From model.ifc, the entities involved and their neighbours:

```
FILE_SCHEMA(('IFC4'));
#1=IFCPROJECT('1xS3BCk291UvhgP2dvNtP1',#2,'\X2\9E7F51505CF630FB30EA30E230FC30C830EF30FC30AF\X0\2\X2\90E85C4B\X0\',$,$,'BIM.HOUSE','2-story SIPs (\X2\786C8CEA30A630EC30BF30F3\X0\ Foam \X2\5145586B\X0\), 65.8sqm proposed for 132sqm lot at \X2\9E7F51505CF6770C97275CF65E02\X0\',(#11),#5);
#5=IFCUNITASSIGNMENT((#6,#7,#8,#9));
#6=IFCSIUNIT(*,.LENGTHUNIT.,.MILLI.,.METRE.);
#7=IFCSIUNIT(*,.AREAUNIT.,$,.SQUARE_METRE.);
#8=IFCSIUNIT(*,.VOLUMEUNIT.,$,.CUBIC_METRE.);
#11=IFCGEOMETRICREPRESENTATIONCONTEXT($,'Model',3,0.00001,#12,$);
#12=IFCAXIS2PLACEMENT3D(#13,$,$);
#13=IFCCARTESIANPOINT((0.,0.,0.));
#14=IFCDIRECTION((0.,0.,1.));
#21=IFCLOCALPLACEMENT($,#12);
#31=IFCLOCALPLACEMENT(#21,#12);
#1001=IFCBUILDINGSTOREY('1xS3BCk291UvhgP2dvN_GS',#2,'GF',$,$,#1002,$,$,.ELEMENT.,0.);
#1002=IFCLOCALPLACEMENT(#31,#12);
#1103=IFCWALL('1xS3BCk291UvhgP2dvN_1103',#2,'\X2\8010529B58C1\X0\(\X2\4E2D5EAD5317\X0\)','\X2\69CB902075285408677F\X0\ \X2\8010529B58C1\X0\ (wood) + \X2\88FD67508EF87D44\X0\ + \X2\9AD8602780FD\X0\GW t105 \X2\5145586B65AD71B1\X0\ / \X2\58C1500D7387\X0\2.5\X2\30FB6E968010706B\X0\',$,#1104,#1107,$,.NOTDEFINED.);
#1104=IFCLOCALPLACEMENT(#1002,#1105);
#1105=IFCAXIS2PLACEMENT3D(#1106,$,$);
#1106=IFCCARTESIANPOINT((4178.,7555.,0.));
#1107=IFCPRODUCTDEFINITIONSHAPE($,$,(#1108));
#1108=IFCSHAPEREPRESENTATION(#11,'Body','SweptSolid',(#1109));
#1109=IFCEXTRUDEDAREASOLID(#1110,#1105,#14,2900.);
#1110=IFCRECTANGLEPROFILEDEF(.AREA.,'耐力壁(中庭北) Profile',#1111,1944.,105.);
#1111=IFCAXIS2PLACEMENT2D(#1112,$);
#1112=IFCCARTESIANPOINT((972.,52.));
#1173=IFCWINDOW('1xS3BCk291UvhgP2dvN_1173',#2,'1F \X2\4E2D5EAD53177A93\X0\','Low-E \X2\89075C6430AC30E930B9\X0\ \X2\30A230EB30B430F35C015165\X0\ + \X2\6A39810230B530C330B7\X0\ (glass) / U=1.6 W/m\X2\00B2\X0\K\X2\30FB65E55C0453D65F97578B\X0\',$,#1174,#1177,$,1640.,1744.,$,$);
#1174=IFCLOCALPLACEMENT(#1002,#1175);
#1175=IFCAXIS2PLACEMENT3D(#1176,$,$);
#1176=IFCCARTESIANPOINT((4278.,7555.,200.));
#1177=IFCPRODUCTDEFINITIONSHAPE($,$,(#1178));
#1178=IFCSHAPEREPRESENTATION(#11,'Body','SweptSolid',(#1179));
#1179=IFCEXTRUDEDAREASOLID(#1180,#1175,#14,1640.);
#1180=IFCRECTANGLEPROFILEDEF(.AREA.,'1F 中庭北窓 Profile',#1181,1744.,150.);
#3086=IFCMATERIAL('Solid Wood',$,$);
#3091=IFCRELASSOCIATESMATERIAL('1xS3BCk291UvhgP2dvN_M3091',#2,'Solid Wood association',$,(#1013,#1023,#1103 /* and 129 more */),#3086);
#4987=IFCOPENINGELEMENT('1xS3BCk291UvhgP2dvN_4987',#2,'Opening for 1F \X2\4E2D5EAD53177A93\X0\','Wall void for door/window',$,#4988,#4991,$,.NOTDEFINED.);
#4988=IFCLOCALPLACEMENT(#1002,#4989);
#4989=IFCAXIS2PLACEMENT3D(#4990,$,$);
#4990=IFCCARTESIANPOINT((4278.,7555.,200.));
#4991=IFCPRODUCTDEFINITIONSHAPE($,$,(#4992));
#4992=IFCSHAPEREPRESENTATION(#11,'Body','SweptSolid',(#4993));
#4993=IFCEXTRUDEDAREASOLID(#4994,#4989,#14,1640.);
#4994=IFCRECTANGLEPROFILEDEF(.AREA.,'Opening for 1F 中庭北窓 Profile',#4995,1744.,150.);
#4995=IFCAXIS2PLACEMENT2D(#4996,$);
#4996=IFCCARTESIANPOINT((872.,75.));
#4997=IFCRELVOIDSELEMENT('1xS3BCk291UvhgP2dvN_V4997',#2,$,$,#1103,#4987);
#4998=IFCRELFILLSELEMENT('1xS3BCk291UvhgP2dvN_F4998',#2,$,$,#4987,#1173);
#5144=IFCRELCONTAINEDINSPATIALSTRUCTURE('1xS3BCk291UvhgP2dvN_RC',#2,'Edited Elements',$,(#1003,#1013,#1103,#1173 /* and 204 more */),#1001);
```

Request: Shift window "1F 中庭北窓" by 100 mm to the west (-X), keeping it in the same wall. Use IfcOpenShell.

```python
import ifcopenshell
import ifcopenshell.api.geometry
import ifcopenshell.util.placement
import ifcopenshell.util.unit

model = ifcopenshell.open("model.ifc")
unit_scale = ifcopenshell.util.unit.calculate_unit_scale(model)

window = model.by_guid("1xS3BCk291UvhgP2dvN_1173")
opening = window.FillsVoids[0].RelatingOpeningElement
wall = opening.VoidsElements[0].RelatingBuildingElement

wall_matrix = ifcopenshell.util.placement.get_local_placement(wall.ObjectPlacement)
shift = wall_matrix[:3, 0] * -0.1 / unit_scale
before = ifcopenshell.util.placement.get_local_placement(window.ObjectPlacement)[:3, 3].copy()

# The window is not placed relative to its opening, so move both.
for product in (opening, window):
    matrix = ifcopenshell.util.placement.get_local_placement(product.ObjectPlacement)
    matrix[:3, 3] += shift
    ifcopenshell.api.geometry.edit_object_placement(model, product=product, matrix=matrix, is_si=False)

after = ifcopenshell.util.placement.get_local_placement(window.ObjectPlacement)[:3, 3]
print("window moved by", (after - before).round(3) + 0.0)

model.write("model_rev.ifc")
```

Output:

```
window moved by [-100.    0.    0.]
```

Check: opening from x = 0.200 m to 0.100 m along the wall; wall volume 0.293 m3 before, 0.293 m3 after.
